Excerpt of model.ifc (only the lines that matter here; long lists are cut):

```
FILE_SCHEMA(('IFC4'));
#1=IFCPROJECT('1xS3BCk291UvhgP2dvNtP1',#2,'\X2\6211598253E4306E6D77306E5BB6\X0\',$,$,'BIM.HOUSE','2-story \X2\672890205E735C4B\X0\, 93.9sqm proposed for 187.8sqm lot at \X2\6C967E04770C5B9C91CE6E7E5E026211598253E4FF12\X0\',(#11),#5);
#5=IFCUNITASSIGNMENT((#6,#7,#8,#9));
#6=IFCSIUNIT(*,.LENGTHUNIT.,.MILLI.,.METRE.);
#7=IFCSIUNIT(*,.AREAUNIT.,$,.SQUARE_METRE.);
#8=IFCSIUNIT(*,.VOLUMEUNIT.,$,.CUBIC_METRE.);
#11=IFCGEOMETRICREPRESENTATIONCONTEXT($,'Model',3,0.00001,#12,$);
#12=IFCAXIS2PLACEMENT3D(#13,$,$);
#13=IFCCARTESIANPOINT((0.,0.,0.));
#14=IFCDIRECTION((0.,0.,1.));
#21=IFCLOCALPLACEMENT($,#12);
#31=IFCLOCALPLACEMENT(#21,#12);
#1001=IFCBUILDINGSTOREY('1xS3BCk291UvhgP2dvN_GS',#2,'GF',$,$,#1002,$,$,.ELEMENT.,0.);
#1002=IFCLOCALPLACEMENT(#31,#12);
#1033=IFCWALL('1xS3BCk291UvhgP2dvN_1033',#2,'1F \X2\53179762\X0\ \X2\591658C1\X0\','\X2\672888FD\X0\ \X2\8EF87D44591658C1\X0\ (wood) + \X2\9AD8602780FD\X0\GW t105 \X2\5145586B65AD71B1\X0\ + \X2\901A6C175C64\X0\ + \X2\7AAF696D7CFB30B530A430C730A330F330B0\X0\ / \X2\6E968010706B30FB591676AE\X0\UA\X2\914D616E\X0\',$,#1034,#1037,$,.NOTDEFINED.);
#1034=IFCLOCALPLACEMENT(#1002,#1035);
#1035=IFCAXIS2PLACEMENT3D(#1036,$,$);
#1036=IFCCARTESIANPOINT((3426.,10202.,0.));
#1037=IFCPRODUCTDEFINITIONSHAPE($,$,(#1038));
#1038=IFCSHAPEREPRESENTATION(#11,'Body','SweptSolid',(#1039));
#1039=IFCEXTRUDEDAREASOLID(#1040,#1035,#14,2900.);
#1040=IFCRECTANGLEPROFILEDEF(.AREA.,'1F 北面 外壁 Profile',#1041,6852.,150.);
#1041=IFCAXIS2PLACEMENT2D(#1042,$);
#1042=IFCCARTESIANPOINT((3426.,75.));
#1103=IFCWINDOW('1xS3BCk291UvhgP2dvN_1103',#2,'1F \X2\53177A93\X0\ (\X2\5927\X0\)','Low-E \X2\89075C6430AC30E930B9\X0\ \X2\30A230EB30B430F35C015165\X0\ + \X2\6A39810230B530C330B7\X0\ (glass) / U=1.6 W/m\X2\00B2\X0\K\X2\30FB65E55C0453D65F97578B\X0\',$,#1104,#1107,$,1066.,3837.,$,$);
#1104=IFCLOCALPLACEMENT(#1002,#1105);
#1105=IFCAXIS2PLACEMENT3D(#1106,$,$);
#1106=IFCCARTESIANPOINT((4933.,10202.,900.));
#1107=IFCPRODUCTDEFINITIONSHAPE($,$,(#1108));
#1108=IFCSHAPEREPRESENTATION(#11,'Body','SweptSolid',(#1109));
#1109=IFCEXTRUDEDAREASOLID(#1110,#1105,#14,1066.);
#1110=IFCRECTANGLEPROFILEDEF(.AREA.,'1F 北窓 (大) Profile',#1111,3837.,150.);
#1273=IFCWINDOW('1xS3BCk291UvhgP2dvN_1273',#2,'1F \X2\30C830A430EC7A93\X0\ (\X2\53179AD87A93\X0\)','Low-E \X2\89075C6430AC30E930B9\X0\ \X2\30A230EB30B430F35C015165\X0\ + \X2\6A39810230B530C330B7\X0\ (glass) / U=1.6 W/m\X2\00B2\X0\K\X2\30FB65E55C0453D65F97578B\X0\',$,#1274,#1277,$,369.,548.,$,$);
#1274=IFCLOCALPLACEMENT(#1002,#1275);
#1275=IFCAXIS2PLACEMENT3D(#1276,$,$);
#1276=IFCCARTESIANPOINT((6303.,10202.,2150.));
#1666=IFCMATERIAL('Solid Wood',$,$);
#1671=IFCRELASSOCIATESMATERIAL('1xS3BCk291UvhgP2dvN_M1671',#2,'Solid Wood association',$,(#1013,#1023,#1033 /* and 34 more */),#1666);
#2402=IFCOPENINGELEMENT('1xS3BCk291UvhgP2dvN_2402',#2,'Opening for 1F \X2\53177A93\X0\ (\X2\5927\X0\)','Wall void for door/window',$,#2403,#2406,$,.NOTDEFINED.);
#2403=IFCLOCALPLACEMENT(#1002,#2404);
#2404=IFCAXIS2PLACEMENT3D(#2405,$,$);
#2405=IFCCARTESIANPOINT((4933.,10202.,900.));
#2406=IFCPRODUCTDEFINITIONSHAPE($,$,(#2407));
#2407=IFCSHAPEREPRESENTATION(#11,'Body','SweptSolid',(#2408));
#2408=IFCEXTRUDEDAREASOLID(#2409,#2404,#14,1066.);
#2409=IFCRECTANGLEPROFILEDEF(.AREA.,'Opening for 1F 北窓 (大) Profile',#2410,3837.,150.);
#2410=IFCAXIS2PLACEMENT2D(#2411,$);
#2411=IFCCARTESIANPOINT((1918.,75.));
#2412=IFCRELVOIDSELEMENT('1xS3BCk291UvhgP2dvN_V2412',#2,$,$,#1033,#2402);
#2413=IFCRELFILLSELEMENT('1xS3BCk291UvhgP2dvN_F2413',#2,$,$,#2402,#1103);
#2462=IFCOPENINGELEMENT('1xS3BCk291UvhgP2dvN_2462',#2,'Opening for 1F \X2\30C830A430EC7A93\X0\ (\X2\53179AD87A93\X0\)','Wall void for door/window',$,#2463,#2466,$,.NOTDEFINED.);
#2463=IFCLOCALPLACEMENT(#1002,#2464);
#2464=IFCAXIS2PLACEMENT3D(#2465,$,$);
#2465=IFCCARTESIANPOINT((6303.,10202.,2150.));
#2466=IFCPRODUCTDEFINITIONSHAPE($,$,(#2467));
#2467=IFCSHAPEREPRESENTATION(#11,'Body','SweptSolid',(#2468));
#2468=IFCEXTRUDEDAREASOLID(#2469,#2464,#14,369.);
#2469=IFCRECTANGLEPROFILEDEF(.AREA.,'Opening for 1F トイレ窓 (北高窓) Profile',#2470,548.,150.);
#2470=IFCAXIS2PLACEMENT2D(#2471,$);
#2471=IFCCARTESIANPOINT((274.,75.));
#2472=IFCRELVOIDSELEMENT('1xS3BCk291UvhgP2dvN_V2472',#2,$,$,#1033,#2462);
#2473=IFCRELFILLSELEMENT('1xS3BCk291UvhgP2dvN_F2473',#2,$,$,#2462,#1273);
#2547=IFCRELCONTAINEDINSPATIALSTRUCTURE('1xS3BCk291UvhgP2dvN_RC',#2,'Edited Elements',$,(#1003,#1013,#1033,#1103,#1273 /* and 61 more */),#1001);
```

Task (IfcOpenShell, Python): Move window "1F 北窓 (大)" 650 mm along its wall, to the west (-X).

```python
import ifcopenshell
import ifcopenshell.api.geometry
import ifcopenshell.util.placement
import ifcopenshell.util.unit

model = ifcopenshell.open("model.ifc")
unit_scale = ifcopenshell.util.unit.calculate_unit_scale(model)

window = model.by_id(1103)
opening = window.FillsVoids[0].RelatingOpeningElement
wall = opening.VoidsElements[0].RelatingBuildingElement

wall_matrix = ifcopenshell.util.placement.get_local_placement(wall.ObjectPlacement)
shift = wall_matrix[:3, 0] * -0.65 / unit_scale
before = ifcopenshell.util.placement.get_local_placement(window.ObjectPlacement)[:3, 3].copy()

# The window is not placed relative to its opening, so move both.
for product in (opening, window):
    matrix = ifcopenshell.util.placement.get_local_placement(product.ObjectPlacement)
    matrix[:3, 3] += shift
    ifcopenshell.api.geometry.edit_object_placement(model, product=product, matrix=matrix, is_si=False)

after = ifcopenshell.util.placement.get_local_placement(window.ObjectPlacement)[:3, 3]
print("window moved by", (after - before).round(3) + 0.0)

model.write("model_edited.ifc")
```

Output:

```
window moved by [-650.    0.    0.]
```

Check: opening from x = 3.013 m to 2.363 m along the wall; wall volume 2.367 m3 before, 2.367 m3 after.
